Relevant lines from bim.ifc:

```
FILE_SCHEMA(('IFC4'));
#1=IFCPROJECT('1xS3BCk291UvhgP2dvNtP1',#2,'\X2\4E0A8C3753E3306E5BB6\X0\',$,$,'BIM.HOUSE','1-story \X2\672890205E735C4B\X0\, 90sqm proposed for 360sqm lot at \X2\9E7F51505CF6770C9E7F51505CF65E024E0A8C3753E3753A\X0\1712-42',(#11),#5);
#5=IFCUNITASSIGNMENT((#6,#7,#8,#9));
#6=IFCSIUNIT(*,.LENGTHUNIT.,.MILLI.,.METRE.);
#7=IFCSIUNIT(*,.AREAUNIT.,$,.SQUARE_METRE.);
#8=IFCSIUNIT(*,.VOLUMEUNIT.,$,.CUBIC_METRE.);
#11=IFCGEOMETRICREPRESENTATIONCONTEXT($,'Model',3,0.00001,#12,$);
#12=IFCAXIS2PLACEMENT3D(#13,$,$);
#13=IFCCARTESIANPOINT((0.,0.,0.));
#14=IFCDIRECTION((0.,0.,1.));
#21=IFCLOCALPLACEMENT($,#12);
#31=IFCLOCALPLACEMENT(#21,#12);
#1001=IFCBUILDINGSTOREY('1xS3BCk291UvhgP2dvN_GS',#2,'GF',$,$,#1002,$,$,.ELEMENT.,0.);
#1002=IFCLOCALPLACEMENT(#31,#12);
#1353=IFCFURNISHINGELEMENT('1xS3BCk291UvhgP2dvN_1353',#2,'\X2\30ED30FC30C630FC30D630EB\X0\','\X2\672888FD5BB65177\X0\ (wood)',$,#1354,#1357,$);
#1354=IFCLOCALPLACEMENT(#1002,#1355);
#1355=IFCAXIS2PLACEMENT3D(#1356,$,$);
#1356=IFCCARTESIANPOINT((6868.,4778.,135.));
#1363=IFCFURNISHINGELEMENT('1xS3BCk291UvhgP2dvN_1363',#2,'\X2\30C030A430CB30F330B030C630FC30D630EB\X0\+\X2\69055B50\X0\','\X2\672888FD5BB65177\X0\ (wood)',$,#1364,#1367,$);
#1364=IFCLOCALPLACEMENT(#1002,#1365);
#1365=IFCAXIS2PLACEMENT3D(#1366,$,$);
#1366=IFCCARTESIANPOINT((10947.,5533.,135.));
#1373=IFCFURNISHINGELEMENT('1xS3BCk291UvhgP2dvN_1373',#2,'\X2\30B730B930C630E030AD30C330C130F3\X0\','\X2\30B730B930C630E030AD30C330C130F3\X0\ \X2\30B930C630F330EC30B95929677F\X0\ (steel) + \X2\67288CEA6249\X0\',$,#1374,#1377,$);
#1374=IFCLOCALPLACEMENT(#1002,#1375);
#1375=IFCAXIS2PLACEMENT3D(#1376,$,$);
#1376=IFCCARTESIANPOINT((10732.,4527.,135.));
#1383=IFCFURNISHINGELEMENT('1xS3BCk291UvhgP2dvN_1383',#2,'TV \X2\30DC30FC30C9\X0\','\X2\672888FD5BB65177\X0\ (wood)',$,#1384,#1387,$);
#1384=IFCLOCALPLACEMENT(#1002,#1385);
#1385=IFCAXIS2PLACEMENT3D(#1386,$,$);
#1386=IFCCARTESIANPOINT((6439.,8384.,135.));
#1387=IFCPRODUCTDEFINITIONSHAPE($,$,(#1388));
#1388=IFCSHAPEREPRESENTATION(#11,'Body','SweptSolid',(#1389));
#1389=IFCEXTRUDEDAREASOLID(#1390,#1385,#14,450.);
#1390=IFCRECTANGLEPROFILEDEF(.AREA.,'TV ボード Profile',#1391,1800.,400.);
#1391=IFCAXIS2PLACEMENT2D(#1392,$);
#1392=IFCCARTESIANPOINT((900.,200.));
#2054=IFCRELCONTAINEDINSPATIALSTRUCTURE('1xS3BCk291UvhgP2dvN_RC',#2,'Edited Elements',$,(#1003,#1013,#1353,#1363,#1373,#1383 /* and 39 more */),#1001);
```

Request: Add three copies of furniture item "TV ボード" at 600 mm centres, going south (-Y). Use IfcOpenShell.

```python
import numpy as np
import ifcopenshell
import ifcopenshell.api.geometry
import ifcopenshell.api.root
import ifcopenshell.util.element
import ifcopenshell.util.placement

model = ifcopenshell.open("bim.ifc")


def reuse_history(source, copy):
    """copy_class also copies each property set's owner history, people and application; keep the originals."""
    for rel in copy.IsDefinedBy:
        if rel.is_a("IfcRelDefinesByProperties") and (history := rel.RelatingPropertyDefinition.OwnerHistory):
            rel.RelatingPropertyDefinition.OwnerHistory = source.OwnerHistory
            ifcopenshell.util.element.remove_deep2(model, history)


source = model.by_guid("1xS3BCk291UvhgP2dvN_1383")
base = ifcopenshell.util.placement.get_local_placement(source.ObjectPlacement)
step = np.array([0.0, -1.0, 0.0]) * 600.0

for i in range(1, 4):
    copy = ifcopenshell.api.root.copy_class(model, product=source)
    copy.Representation = ifcopenshell.util.element.copy_deep(
        model, source.Representation, exclude=["IfcGeometricRepresentationContext", "IfcRepresentationMap"]
    )
    reuse_history(source, copy)
    matrix = base.copy()
    matrix[:3, 3] += i * step
    print("added at", matrix[:3, 3].round(3) + 0.0)
    ifcopenshell.api.geometry.edit_object_placement(model, product=copy, matrix=matrix, is_si=False)

model.write("bim_updated.ifc")
```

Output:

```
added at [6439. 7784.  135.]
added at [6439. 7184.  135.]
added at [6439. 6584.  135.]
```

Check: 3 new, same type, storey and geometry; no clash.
